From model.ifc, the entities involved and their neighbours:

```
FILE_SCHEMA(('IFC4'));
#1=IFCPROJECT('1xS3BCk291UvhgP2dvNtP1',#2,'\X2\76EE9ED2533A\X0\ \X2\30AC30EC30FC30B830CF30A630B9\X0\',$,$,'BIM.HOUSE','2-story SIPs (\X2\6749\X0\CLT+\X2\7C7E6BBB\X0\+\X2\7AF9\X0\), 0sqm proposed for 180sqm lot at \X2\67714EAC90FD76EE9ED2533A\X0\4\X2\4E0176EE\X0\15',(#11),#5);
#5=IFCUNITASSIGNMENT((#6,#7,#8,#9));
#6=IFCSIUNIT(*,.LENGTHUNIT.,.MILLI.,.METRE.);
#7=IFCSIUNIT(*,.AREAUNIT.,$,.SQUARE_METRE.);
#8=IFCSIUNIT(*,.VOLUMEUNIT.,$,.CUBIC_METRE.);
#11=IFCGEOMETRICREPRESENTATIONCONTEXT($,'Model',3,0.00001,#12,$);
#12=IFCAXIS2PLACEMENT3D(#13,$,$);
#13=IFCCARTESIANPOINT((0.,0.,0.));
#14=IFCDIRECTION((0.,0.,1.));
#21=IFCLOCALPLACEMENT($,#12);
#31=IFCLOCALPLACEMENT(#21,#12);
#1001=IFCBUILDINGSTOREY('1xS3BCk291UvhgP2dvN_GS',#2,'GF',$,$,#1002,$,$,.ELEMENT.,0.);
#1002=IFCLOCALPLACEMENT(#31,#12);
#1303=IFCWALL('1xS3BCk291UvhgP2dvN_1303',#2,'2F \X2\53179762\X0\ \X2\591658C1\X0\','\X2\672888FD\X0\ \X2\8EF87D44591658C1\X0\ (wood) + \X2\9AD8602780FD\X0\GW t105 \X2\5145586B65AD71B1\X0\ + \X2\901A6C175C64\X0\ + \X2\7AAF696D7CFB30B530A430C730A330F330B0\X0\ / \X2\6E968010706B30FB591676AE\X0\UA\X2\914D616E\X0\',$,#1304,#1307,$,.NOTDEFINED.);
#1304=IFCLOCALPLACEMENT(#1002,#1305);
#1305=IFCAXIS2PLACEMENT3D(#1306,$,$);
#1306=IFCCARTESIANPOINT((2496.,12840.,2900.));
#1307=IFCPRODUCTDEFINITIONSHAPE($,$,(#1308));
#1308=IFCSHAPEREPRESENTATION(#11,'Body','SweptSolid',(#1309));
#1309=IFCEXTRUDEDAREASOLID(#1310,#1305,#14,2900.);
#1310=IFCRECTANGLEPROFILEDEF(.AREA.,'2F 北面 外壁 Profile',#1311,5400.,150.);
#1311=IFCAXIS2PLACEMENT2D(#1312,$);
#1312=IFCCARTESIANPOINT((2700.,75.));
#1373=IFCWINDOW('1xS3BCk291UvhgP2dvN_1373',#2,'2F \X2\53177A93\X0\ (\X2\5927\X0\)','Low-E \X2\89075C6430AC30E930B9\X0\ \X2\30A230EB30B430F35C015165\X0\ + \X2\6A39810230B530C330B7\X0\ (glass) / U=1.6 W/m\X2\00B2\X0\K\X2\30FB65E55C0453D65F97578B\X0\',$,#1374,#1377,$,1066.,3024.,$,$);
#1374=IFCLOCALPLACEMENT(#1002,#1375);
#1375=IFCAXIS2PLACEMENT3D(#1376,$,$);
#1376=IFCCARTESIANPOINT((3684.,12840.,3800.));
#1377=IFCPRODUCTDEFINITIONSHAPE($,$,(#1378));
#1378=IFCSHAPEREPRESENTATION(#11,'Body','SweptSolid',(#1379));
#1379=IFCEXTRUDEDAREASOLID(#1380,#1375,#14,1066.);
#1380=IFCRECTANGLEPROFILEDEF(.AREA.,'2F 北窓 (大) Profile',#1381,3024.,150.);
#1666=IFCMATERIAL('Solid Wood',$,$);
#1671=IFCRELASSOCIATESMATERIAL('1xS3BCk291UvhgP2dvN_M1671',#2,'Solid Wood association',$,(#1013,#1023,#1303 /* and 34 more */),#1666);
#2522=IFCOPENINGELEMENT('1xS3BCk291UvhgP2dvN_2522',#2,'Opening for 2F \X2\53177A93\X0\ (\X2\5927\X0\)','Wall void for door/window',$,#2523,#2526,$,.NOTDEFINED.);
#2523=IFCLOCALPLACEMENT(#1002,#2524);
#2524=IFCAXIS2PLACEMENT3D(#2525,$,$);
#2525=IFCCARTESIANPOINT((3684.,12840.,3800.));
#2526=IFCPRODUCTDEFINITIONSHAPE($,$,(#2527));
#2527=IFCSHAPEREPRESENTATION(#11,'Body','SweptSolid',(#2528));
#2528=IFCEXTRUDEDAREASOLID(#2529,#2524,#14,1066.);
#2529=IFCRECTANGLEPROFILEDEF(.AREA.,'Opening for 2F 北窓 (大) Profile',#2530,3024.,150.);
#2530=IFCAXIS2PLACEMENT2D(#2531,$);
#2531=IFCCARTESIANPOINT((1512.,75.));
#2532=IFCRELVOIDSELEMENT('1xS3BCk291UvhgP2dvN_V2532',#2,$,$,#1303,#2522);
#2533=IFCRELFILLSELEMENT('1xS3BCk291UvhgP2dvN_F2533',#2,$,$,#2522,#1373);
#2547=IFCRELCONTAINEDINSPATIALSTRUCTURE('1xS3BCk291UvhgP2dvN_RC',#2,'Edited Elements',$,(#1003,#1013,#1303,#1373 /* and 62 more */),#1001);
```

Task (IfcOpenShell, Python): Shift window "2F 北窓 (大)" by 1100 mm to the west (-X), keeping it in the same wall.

```python
import ifcopenshell
import ifcopenshell.api.geometry
import ifcopenshell.util.placement
import ifcopenshell.util.unit

model = ifcopenshell.open("model.ifc")
unit_scale = ifcopenshell.util.unit.calculate_unit_scale(model)

window = model.by_guid("1xS3BCk291UvhgP2dvN_1373")
opening = window.FillsVoids[0].RelatingOpeningElement
wall = opening.VoidsElements[0].RelatingBuildingElement

wall_matrix = ifcopenshell.util.placement.get_local_placement(wall.ObjectPlacement)
shift = wall_matrix[:3, 0] * -1.1 / unit_scale
before = ifcopenshell.util.placement.get_local_placement(window.ObjectPlacement)[:3, 3].copy()

# The window is not placed relative to its opening, so move both.
for product in (opening, window):
    matrix = ifcopenshell.util.placement.get_local_placement(product.ObjectPlacement)
    matrix[:3, 3] += shift
    ifcopenshell.api.geometry.edit_object_placement(model, product=product, matrix=matrix, is_si=False)

after = ifcopenshell.util.placement.get_local_placement(window.ObjectPlacement)[:3, 3]
print("window moved by", (after - before).round(3) + 0.0)

model.write("model-out.ifc")
```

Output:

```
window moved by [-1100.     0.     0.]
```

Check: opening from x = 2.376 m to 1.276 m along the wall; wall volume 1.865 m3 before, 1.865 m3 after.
